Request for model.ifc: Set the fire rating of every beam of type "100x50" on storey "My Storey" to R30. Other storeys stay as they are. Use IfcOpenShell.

First a look at what the model holds.

```python
import ifcopenshell
import ifcopenshell.util.element

model = ifcopenshell.open("model.ifc")
print(model.schema)
storey = next(s for s in model.by_type("IfcBuildingStorey") if s.Name == "My Storey")
beams = [e for e in ifcopenshell.util.element.get_decomposition(storey) if e.is_a("IfcBeam")]
seen = {}
for e in beams:
    element_type = ifcopenshell.util.element.get_type(e)
    key = (element_type.Name if element_type != e and element_type else None, ifcopenshell.util.element.get_pset(e, "Pset_BeamCommon", "FireRating"))
    seen[key] = seen.get(key, 0) + 1
for (name, value), count in sorted(seen.items(), key=str):
    print(count, "x", name, "|", value)
```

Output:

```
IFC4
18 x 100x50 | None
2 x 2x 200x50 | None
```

```python
import ifcopenshell
import ifcopenshell.api.pset
import ifcopenshell.util.element

model = ifcopenshell.open("model.ifc")

storey = next(s for s in model.by_type("IfcBuildingStorey") if s.Name == "My Storey")
beams = [e for e in ifcopenshell.util.element.get_decomposition(storey) if e.is_a("IfcBeam")]

count = 0
for e in beams:
    element_type = ifcopenshell.util.element.get_type(e)
    if element_type in (None, e) or element_type.Name != "100x50":
        continue
    # add_pset returns the element's existing set when there is one.
    pset = ifcopenshell.api.pset.add_pset(model, product=e, name="Pset_BeamCommon")
    ifcopenshell.api.pset.edit_pset(model, pset=pset, properties={"FireRating": "R30"})
    count += 1

print(count, "beams updated")

model.write("model-out.ifc")
```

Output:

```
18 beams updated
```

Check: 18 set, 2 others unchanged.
